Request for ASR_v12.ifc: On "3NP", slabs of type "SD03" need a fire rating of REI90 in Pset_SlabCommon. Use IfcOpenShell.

First a look at what the model holds.

```python
import ifcopenshell
import ifcopenshell.util.element

model = ifcopenshell.open("ASR_v12.ifc")
print(model.schema)
storey = next(s for s in model.by_type("IfcBuildingStorey") if s.Name == "3NP")
slabs = [e for e in ifcopenshell.util.element.get_decomposition(storey) if e.is_a("IfcSlab")]
seen = {}
for e in slabs:
    element_type = ifcopenshell.util.element.get_type(e)
    key = (element_type.Name if element_type != e and element_type else None, ifcopenshell.util.element.get_pset(e, "Pset_SlabCommon", "FireRating"))
    seen[key] = seen.get(key, 0) + 1
for (name, value), count in sorted(seen.items(), key=str):
    print(count, "x", name, "|", value)
```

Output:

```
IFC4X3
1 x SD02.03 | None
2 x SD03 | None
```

```python
import ifcopenshell
import ifcopenshell.api.pset
import ifcopenshell.util.element

model = ifcopenshell.open("ASR_v12.ifc")

storey = next(s for s in model.by_type("IfcBuildingStorey") if s.Name == "3NP")
slabs = [e for e in ifcopenshell.util.element.get_decomposition(storey) if e.is_a("IfcSlab")]

count = 0
for e in slabs:
    element_type = ifcopenshell.util.element.get_type(e)
    if element_type in (None, e) or element_type.Name != "SD03":
        continue
    # add_pset returns the element's existing set when there is one.
    pset = ifcopenshell.api.pset.add_pset(model, product=e, name="Pset_SlabCommon")
    ifcopenshell.api.pset.edit_pset(model, pset=pset, properties={"FireRating": "REI90"})
    count += 1

print(count, "slabs updated")

model.write("ASR_v12_rev.ifc")
```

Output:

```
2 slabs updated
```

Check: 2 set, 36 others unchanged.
